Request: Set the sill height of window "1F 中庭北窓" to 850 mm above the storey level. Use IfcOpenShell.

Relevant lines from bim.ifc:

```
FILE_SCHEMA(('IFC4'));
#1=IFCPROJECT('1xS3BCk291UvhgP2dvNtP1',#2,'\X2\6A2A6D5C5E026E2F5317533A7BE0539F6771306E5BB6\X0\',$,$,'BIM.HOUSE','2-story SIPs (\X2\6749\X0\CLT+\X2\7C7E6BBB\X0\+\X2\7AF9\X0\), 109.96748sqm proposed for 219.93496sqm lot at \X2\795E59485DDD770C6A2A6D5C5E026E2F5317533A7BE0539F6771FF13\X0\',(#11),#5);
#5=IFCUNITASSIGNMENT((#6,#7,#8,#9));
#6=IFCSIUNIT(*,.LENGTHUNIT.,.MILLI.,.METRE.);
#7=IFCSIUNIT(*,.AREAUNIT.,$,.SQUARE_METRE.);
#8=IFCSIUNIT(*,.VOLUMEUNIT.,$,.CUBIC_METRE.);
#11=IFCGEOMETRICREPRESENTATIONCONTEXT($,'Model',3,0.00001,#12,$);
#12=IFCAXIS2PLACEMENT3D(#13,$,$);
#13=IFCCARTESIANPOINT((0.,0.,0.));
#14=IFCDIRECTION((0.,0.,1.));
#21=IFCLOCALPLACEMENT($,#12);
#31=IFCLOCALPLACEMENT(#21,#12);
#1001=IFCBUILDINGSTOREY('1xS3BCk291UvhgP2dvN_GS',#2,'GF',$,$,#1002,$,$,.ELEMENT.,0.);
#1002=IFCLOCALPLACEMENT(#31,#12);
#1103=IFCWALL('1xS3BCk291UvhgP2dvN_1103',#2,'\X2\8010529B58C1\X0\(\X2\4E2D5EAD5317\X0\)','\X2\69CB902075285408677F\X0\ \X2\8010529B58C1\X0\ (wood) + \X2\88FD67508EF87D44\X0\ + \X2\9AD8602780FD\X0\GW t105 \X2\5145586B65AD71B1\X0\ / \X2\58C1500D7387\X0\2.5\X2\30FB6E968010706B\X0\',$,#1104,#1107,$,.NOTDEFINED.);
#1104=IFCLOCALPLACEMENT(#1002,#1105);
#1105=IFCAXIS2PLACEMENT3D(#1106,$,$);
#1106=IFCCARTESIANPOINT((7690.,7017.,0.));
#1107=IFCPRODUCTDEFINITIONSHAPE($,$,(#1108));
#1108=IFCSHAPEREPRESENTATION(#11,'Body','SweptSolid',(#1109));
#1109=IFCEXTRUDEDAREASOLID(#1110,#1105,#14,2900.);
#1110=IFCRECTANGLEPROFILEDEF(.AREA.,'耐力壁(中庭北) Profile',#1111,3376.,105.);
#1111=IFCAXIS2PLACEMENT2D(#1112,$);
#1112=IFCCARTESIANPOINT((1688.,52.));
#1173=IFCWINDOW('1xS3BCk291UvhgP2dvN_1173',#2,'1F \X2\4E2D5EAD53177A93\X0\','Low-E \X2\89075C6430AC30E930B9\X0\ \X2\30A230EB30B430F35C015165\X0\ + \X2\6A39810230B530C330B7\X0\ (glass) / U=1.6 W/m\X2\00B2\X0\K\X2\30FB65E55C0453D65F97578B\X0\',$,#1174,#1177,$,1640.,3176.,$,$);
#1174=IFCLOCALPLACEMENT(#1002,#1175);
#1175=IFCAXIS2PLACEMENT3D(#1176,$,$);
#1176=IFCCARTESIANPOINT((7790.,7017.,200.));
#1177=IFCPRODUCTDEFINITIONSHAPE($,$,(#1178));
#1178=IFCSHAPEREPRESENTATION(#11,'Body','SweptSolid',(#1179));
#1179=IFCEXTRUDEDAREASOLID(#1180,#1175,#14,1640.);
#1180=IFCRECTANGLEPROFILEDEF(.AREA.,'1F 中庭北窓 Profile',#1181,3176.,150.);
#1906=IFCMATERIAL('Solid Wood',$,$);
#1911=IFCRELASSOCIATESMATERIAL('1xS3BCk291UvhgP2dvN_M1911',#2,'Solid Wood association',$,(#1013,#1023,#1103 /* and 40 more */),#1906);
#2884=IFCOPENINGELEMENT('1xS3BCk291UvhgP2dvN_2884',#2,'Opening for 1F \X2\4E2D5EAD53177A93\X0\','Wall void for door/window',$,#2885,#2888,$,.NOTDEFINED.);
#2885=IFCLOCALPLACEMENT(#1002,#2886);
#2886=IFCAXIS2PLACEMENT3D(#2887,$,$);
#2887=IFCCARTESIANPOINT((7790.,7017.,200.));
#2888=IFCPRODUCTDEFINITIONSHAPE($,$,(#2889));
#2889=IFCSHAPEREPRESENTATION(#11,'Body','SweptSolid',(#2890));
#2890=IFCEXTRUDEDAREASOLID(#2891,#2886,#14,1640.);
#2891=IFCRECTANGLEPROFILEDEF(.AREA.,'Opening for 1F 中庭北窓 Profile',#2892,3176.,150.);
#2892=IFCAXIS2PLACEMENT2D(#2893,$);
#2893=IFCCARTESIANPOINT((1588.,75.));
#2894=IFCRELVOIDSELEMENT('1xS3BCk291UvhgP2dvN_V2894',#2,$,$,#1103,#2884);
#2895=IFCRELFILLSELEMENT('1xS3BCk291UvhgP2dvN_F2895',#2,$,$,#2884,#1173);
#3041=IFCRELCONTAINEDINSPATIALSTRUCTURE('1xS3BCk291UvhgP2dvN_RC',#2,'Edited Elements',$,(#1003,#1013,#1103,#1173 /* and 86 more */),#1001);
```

```python
import numpy as np
import ifcopenshell
import ifcopenshell.api.geometry
import ifcopenshell.geom
import ifcopenshell.util.element
import ifcopenshell.util.placement
import ifcopenshell.util.shape
import ifcopenshell.util.unit

model = ifcopenshell.open("bim.ifc")
unit_scale = ifcopenshell.util.unit.calculate_unit_scale(model)

window = model.by_id(1173)
opening = window.FillsVoids[0].RelatingOpeningElement
storey = ifcopenshell.util.element.get_container(window, ifc_class="IfcBuildingStorey")
level = ifcopenshell.util.placement.get_local_placement(storey.ObjectPlacement)[2, 3]

# The opening's origin need not be at the sill, so measure its lowest point.
shape = ifcopenshell.geom.create_shape(ifcopenshell.geom.settings(), opening)
bottom = ifcopenshell.util.shape.get_shape_bottom_elevation(shape, shape.geometry) / unit_scale
dz = level + 850.0 - bottom

shift = np.array([0.0, 0.0, dz])
# The window is not placed relative to its opening, so move both.
for product in (opening, window):
    matrix = ifcopenshell.util.placement.get_local_placement(product.ObjectPlacement)
    matrix[:3, 3] += shift
    ifcopenshell.api.geometry.edit_object_placement(model, product=product, matrix=matrix, is_si=False)

print(f"moved by {dz * unit_scale:+.3f} m")

model.write("bim_updated.ifc")
```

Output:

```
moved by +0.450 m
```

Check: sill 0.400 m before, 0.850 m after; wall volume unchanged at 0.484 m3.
